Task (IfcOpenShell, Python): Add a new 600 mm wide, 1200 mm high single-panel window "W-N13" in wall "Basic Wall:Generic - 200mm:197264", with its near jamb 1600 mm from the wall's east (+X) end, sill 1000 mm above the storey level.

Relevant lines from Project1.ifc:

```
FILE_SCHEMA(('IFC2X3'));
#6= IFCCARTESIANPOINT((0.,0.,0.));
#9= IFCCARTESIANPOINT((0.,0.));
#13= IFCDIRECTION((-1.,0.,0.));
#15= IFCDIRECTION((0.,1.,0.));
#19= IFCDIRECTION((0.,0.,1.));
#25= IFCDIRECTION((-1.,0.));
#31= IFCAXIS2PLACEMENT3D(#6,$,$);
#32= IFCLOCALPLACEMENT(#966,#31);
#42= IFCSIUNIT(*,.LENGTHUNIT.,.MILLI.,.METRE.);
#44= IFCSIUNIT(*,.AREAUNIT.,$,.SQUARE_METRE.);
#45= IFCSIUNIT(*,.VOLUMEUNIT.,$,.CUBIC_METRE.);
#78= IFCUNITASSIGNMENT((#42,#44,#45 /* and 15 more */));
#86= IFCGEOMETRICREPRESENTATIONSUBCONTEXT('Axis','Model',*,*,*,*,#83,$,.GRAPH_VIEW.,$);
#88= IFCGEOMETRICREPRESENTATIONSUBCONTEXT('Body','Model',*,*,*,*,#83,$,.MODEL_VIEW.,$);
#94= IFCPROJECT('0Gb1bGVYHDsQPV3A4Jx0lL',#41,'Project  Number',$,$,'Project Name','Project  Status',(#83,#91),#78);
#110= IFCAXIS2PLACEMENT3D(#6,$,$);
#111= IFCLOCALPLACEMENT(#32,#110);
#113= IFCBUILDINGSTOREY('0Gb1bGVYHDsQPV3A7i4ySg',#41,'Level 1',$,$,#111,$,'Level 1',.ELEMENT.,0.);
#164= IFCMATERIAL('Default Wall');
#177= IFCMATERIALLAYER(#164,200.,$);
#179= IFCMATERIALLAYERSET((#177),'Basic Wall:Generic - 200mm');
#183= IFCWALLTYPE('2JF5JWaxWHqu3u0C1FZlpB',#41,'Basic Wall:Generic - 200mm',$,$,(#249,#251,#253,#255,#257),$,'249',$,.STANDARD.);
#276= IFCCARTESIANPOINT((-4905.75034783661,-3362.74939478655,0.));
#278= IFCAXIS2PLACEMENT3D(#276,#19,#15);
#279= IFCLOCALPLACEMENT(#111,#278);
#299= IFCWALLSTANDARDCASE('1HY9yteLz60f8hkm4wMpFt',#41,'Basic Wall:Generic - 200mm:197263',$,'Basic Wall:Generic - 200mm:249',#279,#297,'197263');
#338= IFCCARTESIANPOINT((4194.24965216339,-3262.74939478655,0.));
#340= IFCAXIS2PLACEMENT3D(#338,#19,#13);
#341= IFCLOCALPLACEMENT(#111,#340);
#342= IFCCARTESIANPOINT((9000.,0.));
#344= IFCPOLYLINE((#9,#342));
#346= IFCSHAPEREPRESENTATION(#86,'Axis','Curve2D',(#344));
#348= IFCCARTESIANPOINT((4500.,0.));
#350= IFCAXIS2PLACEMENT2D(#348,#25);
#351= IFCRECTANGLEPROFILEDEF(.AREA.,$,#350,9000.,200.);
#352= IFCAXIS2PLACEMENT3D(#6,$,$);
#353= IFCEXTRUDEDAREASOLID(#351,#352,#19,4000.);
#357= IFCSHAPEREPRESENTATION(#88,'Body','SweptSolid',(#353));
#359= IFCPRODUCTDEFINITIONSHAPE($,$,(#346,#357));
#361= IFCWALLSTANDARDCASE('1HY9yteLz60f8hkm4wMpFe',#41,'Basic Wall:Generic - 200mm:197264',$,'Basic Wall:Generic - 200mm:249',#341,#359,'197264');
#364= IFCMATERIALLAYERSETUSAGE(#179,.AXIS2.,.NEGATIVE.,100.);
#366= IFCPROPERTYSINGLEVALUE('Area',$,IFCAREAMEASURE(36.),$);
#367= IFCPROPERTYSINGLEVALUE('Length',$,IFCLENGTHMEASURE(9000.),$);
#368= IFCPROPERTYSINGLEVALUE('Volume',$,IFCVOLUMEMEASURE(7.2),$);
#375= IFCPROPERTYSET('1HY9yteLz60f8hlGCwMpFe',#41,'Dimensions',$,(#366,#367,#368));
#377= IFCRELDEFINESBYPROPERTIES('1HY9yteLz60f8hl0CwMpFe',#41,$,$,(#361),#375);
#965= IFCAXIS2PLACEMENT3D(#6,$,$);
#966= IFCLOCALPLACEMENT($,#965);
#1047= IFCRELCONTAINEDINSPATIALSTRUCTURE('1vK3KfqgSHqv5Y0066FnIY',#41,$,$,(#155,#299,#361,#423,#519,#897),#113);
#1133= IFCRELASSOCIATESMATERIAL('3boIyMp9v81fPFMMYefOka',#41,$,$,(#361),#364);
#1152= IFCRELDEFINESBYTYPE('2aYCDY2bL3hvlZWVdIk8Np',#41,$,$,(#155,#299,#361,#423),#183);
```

```python
import numpy as np
import ifcopenshell
import ifcopenshell.api.feature
import ifcopenshell.api.geometry
import ifcopenshell.api.pset
import ifcopenshell.api.root
import ifcopenshell.api.spatial
import ifcopenshell.api.type
import ifcopenshell.geom
import ifcopenshell.util.element
import ifcopenshell.util.placement
import ifcopenshell.util.representation
import ifcopenshell.util.shape
import ifcopenshell.util.unit

model = ifcopenshell.open("Project1.ifc")
unit_scale = ifcopenshell.util.unit.calculate_unit_scale(model)
area_scale = ifcopenshell.util.unit.calculate_unit_scale(model, "AREAUNIT")
volume_scale = ifcopenshell.util.unit.calculate_unit_scale(model, "VOLUMEUNIT")
settings = ifcopenshell.geom.settings()


def volume(element):
    """Net volume in cubic metres, openings subtracted."""
    shape = ifcopenshell.geom.create_shape(settings, element)
    return ifcopenshell.util.shape.get_volume(shape.geometry)


wall = model.by_guid("1HY9yteLz60f8hkm4wMpFe")
storey = ifcopenshell.util.element.get_container(wall, ifc_class="IfcBuildingStorey")
context = ifcopenshell.util.representation.get_context(model, "Model", "Body", "MODEL_VIEW")
before = volume(wall)

width, height, from_end, sill = 0.6, 1.2, 1.6, 1  # metres

# The wall runs along its own X axis, and the end named is its -X end.
wall_shape = ifcopenshell.geom.create_shape(settings, wall)
x, y, z = ifcopenshell.util.shape.get_vertices(wall_shape.geometry).T
start = x.min() + from_end
face, thickness = float(y.min()), float(y.max() - y.min())
wall_matrix = ifcopenshell.util.placement.get_local_placement(wall.ObjectPlacement)
level = ifcopenshell.util.placement.get_local_placement(storey.ObjectPlacement)[2, 3]


def in_wall(x, y):
    """Placement at x, y metres in the wall's axes, at sill height."""
    matrix = wall_matrix.copy()
    matrix[:, 3] = wall_matrix @ np.array([x / unit_scale, y / unit_scale, 0.0, 1.0])
    matrix[2, 3] = level + sill / unit_scale
    return matrix


# Opening: a box that overshoots both wall faces by 50 mm.
opening = ifcopenshell.api.root.create_entity(model, ifc_class="IfcOpeningElement")
box = ifcopenshell.api.geometry.add_wall_representation(
    model, context=context, length=width, height=height, thickness=thickness + 0.1
)
ifcopenshell.api.geometry.assign_representation(model, product=opening, representation=box)
ifcopenshell.api.geometry.edit_object_placement(model, product=opening, matrix=in_wall(start, face - 0.05), is_si=False)
ifcopenshell.api.feature.add_feature(model, feature=opening, element=wall)

window = ifcopenshell.api.root.create_entity(model, ifc_class="IfcWindow", name="W-N13")
window.OverallWidth, window.OverallHeight = width / unit_scale, height / unit_scale
body = ifcopenshell.api.geometry.add_window_representation(
    model,
    context=context,
    overall_width=window.OverallWidth,
    overall_height=window.OverallHeight,
    partition_type="SINGLE_PANEL",
)
ifcopenshell.api.geometry.assign_representation(model, product=window, representation=body)
ifcopenshell.api.spatial.assign_container(model, products=[window], relating_structure=storey)
fills = ifcopenshell.api.feature.add_filling(model, opening=opening, element=window)
fills.OwnerHistory = window.OwnerHistory  # required in IFC2X3

# IFC2X3 keeps the operation on the window style.
style = ifcopenshell.api.root.create_entity(model, ifc_class="IfcWindowStyle", name="W-N13")
style.OperationType, style.ConstructionType = "SINGLE_PANEL", "NOTDEFINED"
style.ParameterTakesPrecedence = style.Sizeable = False
ifcopenshell.api.type.assign_type(model, related_objects=[window], relating_type=style)

# Centre the window in the wall's thickness.
ifcopenshell.api.geometry.edit_object_placement(model, product=window, matrix=in_wall(start, face), is_si=False)
window_shape = ifcopenshell.geom.create_shape(settings, window)
depth = ifcopenshell.util.shape.get_vertices(window_shape.geometry)[:, 1]
offset = face + thickness / 2 - (depth.min() + depth.max()) / 2
ifcopenshell.api.geometry.edit_object_placement(model, product=window, matrix=in_wall(start, offset), is_si=False)

after = volume(wall)

# Update the wall's stored quantities.
pset = model.by_id(ifcopenshell.util.element.get_pset(wall, "Dimensions", should_inherit=False)["id"])
ifcopenshell.api.pset.edit_pset(model, pset=pset, properties={
    "Area": model.create_entity("IfcAreaMeasure", after / thickness / area_scale),
    "Volume": model.create_entity("IfcVolumeMeasure", after / volume_scale),
})

print(f"wall volume {before:.3f} -> {after:.3f} m3")

model.write("Project1_updated.ifc")
```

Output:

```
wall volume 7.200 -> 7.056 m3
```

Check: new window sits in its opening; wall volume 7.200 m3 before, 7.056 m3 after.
